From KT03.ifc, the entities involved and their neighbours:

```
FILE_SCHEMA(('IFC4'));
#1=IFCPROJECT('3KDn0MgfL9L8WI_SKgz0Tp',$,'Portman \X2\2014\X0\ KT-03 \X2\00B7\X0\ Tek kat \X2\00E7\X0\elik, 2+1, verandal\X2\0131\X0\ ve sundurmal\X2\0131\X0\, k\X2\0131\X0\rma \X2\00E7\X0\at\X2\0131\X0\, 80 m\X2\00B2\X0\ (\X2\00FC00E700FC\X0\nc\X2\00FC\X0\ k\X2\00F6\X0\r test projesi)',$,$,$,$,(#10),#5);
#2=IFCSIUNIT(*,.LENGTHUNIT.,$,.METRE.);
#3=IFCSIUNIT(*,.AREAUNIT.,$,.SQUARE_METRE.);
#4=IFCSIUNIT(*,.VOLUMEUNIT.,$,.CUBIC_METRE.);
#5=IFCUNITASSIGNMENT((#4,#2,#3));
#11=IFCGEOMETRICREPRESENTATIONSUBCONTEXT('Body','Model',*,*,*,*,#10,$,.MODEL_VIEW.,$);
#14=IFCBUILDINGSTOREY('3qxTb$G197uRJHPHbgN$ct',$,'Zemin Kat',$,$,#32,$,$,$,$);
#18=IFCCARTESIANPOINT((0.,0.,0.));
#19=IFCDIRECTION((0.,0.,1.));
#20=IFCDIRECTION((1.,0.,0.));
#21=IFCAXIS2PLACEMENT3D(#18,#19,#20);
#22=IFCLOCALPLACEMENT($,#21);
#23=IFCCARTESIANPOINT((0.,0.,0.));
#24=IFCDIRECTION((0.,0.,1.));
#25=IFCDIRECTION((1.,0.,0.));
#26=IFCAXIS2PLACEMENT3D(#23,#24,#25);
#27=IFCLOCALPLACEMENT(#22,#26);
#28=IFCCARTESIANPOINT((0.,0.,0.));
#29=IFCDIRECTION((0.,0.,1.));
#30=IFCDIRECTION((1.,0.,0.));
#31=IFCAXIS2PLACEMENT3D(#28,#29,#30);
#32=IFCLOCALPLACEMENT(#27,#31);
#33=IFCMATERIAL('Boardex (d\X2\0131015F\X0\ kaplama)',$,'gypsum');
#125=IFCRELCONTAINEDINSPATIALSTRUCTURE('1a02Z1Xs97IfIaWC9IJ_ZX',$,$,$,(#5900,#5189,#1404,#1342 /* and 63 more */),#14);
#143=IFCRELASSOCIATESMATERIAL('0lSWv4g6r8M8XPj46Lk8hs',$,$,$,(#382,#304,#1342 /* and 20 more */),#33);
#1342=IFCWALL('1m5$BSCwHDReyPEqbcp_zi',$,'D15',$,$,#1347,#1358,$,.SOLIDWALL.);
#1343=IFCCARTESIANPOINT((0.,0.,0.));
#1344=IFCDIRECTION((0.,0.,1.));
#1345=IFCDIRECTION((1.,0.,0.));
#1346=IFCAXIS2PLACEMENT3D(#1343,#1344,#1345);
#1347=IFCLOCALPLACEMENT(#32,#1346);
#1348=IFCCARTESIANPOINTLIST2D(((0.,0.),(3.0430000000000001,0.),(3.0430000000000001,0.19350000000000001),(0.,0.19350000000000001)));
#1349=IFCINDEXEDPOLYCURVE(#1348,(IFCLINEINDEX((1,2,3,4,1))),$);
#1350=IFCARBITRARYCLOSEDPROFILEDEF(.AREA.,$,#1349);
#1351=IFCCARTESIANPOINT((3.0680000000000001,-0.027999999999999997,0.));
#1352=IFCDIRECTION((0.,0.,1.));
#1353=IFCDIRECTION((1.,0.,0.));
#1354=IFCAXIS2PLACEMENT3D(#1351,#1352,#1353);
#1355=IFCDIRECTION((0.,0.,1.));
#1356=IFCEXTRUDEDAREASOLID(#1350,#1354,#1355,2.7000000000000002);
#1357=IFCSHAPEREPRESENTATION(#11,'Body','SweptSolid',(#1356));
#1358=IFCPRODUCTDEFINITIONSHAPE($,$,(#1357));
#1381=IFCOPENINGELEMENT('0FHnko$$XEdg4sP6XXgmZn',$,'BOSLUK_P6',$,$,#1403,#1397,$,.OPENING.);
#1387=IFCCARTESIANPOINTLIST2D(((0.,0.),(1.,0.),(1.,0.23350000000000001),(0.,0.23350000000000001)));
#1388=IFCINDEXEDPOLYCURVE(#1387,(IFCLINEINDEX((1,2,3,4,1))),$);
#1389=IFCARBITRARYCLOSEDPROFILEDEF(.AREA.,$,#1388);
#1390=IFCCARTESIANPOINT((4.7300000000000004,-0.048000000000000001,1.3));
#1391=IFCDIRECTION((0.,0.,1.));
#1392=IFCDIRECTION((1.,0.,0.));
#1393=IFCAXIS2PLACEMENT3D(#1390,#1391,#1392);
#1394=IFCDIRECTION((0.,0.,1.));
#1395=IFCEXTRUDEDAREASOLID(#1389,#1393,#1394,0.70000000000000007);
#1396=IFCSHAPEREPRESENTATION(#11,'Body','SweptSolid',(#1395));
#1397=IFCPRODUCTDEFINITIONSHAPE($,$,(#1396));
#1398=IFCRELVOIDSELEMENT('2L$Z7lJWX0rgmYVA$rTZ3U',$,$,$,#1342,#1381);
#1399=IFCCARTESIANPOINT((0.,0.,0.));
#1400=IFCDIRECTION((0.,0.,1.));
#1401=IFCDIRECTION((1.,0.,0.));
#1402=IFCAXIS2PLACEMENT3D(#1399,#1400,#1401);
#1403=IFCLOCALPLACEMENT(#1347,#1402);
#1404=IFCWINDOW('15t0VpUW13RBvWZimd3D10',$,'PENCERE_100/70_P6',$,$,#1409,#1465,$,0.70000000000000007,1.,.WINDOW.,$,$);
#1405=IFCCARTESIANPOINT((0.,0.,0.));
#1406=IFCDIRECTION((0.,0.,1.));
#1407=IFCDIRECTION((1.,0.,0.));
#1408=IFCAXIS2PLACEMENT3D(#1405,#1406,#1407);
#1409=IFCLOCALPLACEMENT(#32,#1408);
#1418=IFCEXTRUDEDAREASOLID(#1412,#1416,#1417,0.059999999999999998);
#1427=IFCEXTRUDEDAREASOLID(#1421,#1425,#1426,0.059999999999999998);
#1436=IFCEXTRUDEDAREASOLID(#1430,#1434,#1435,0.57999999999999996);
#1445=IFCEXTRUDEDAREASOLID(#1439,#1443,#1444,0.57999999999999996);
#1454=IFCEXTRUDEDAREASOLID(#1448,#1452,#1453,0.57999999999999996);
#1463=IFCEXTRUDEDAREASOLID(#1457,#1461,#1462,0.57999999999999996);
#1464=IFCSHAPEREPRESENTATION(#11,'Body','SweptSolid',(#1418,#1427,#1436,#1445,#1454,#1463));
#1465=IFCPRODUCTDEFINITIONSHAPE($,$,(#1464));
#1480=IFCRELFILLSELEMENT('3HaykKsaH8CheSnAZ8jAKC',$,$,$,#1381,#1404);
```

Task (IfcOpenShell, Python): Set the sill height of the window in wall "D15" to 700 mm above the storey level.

```python
import numpy as np
import ifcopenshell
import ifcopenshell.api.geometry
import ifcopenshell.geom
import ifcopenshell.util.element
import ifcopenshell.util.placement
import ifcopenshell.util.shape
import ifcopenshell.util.unit

model = ifcopenshell.open("KT03.ifc")
unit_scale = ifcopenshell.util.unit.calculate_unit_scale(model)

window = model.by_guid("15t0VpUW13RBvWZimd3D10")
opening = window.FillsVoids[0].RelatingOpeningElement
storey = ifcopenshell.util.element.get_container(window, ifc_class="IfcBuildingStorey")
level = ifcopenshell.util.placement.get_local_placement(storey.ObjectPlacement)[2, 3]

# The opening's origin need not be at the sill, so measure its lowest point.
shape = ifcopenshell.geom.create_shape(ifcopenshell.geom.settings(), opening)
bottom = ifcopenshell.util.shape.get_shape_bottom_elevation(shape, shape.geometry) / unit_scale
dz = level + 0.7 - bottom

shift = np.array([0.0, 0.0, dz])
# The window is not placed relative to its opening, so move both.
for product in (opening, window):
    matrix = ifcopenshell.util.placement.get_local_placement(product.ObjectPlacement)
    matrix[:3, 3] += shift
    ifcopenshell.api.geometry.edit_object_placement(model, product=product, matrix=matrix, is_si=False)

print(f"moved by {dz * unit_scale:+.3f} m")

model.write("KT03_v2.ifc")
```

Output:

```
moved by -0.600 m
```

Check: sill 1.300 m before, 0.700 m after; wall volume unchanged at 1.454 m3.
